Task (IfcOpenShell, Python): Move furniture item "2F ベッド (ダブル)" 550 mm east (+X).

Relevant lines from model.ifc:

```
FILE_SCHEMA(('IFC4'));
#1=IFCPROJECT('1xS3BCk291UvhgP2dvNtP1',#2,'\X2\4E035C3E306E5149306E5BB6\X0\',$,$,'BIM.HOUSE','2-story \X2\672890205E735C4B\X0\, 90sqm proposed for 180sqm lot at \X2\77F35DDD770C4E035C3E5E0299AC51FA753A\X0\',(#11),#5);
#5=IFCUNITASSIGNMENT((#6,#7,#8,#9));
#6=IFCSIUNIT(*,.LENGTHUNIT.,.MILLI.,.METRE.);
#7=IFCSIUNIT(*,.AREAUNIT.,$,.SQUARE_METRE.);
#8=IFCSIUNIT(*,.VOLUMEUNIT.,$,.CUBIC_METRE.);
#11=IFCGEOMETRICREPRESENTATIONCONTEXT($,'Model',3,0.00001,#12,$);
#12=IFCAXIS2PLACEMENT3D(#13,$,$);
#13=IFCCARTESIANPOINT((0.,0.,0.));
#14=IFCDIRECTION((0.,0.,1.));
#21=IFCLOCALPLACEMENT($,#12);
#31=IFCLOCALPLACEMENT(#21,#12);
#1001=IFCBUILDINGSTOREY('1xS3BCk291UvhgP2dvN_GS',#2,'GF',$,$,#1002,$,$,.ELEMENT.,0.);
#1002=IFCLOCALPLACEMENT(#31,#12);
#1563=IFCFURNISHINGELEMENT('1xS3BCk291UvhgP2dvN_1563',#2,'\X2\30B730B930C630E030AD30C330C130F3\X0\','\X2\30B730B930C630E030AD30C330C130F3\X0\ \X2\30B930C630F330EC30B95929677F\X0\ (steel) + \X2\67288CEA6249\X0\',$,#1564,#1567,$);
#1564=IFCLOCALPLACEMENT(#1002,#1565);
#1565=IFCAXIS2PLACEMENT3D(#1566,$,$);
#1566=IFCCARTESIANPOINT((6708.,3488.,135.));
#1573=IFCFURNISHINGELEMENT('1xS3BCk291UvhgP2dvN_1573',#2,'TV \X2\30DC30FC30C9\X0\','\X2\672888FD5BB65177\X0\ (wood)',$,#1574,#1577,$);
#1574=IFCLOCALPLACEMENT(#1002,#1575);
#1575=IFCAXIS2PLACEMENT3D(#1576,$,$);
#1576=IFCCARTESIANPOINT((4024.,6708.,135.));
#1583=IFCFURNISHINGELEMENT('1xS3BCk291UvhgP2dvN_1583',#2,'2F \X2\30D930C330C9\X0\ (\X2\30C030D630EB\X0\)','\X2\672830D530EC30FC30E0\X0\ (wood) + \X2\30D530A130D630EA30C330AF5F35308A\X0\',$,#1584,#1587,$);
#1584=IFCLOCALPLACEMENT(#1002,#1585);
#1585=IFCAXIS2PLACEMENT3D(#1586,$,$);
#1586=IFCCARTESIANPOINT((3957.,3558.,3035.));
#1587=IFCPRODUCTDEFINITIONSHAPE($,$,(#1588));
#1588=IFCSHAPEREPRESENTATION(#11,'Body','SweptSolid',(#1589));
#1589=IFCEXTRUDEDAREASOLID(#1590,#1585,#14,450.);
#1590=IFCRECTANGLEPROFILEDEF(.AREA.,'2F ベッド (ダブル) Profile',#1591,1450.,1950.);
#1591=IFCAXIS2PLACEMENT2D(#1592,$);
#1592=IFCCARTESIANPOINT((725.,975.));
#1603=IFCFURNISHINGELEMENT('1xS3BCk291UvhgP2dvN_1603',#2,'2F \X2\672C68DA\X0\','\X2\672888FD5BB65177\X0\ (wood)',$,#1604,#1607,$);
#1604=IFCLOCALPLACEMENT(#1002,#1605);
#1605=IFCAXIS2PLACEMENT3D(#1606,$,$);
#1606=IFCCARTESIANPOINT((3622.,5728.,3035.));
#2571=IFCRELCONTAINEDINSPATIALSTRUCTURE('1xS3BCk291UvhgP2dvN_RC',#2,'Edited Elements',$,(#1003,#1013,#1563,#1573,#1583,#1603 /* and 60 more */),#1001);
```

```python
import ifcopenshell
import ifcopenshell.api.geometry
import ifcopenshell.util.placement

model = ifcopenshell.open("model.ifc")

item = model.by_guid("1xS3BCk291UvhgP2dvN_1583")
matrix = ifcopenshell.util.placement.get_local_placement(item.ObjectPlacement)
matrix[0, 3] += 550.0
ifcopenshell.api.geometry.edit_object_placement(model, product=item, matrix=matrix, is_si=False)

print(ifcopenshell.util.placement.get_local_placement(item.ObjectPlacement).round(3) + 0.0)

model.write("model_edited.ifc")
```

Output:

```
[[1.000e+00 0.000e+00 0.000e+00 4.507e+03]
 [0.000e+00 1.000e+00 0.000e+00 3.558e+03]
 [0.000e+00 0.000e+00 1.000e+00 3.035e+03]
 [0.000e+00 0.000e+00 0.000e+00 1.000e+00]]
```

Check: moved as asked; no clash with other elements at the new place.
